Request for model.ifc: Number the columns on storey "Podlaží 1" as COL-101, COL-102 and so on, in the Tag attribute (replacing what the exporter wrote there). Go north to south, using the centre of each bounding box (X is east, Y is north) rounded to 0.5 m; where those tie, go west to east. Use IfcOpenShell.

First a look at what the model holds.

```python
import ifcopenshell
import ifcopenshell.util.element
import ifcopenshell.util.placement

model = ifcopenshell.open("model.ifc")
print(model.schema)
storey = next(s for s in model.by_type("IfcBuildingStorey") if s.Name == "Podlaží 1")
columns = [e for e in ifcopenshell.util.element.get_decomposition(storey) if e.is_a("IfcColumn")]
for e in sorted(columns, key=lambda e: e.id()):
    origin = ifcopenshell.util.placement.get_local_placement(e.ObjectPlacement)[:3, 3]
    print(e.id(), e.Tag, e.Name, origin.round(2) + 0.0, sep=" | ")
```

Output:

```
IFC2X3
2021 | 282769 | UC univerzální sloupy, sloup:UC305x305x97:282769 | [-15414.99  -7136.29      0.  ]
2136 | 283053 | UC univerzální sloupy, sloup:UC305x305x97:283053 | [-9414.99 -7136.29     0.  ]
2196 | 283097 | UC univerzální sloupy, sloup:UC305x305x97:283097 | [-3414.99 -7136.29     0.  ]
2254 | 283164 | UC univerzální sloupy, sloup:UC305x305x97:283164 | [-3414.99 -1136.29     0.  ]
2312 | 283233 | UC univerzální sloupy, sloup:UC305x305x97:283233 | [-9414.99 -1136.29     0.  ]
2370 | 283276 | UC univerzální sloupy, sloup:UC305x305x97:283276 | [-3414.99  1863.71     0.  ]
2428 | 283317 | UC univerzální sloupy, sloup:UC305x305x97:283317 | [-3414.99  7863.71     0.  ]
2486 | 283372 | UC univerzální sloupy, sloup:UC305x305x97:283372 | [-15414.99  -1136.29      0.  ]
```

```python
import ifcopenshell
import ifcopenshell.geom
import ifcopenshell.util.element
import ifcopenshell.util.shape

model = ifcopenshell.open("model.ifc")
settings = ifcopenshell.geom.settings()
settings.set("use-world-coords", True)


def centre(element):
    shape = ifcopenshell.geom.create_shape(settings, element)
    return ifcopenshell.util.shape.get_bbox_centroid(shape.geometry)


storey = next(s for s in model.by_type("IfcBuildingStorey") if s.Name == "Podlaží 1")
columns = [e for e in ifcopenshell.util.element.get_decomposition(storey) if e.is_a("IfcColumn")]

# Insertion points can sit at a corner or the storey origin, so sort by the geometry (in metres).
centres = {e: centre(e) for e in columns}
columns.sort(key=lambda e: (-round(centres[e][1] / 0.5), centres[e][0]))

for i, e in enumerate(columns, start=1):
    number = f"COL-1{i:02d}"
    e.Tag = number
    print(e.id(), number)

model.write("model_v2.ifc")
```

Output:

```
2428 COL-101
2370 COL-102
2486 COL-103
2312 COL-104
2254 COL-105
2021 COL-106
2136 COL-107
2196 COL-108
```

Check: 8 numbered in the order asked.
